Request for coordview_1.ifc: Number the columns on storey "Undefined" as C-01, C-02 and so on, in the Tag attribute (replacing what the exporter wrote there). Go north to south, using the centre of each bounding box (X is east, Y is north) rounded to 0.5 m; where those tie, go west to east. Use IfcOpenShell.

First a look at what the model holds.

```python
import ifcopenshell
import ifcopenshell.util.element
import ifcopenshell.util.placement

model = ifcopenshell.open("coordview_1.ifc")
print(model.schema)
storey = next(s for s in model.by_type("IfcBuildingStorey") if s.Name == "Undefined")
columns = [e for e in ifcopenshell.util.element.get_decomposition(storey) if e.is_a("IfcColumn")]
for e in sorted(columns, key=lambda e: e.id()):
    origin = ifcopenshell.util.placement.get_local_placement(e.ObjectPlacement)[:3, 3]
    print(e.id(), e.Tag, e.Name, origin.round(2) + 0.0, sep=" | ")
```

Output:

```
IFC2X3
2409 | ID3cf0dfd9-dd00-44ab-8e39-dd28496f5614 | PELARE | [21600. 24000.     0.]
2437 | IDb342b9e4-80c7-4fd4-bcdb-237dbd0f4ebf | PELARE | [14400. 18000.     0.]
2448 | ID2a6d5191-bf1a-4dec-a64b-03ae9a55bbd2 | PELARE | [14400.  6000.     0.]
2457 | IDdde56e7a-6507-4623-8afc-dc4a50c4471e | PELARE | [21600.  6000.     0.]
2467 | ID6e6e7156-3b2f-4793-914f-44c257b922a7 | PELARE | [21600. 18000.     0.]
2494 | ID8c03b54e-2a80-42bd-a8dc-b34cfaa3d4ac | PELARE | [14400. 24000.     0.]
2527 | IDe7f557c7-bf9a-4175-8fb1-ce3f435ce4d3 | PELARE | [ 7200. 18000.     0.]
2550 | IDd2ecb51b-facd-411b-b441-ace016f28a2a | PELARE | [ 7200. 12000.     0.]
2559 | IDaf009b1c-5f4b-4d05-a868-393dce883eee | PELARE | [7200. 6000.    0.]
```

```python
import ifcopenshell
import ifcopenshell.geom
import ifcopenshell.util.element
import ifcopenshell.util.shape

model = ifcopenshell.open("coordview_1.ifc")
settings = ifcopenshell.geom.settings()
settings.set("use-world-coords", True)


def centre(element):
    shape = ifcopenshell.geom.create_shape(settings, element)
    return ifcopenshell.util.shape.get_bbox_centroid(shape.geometry)


storey = next(s for s in model.by_type("IfcBuildingStorey") if s.Name == "Undefined")
columns = [e for e in ifcopenshell.util.element.get_decomposition(storey) if e.is_a("IfcColumn")]

# Insertion points can sit at a corner or the storey origin, so sort by the geometry (in metres).
centres = {e: centre(e) for e in columns}
columns.sort(key=lambda e: (-round(centres[e][1] / 0.5), centres[e][0]))

for i, e in enumerate(columns, start=1):
    number = f"C-{i:02d}"
    e.Tag = number
    print(e.id(), number)

model.write("coordview_1_v2.ifc")
```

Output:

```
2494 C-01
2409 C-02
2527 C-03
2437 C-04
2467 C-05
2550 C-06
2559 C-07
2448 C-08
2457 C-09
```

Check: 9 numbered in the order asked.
